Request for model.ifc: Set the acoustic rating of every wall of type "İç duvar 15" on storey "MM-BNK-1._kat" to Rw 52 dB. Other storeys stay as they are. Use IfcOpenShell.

First a look at what the model holds.

```python
import ifcopenshell
import ifcopenshell.util.element

model = ifcopenshell.open("model.ifc")
print(model.schema)
storey = next(s for s in model.by_type("IfcBuildingStorey") if s.Name == "MM-BNK-1._kat")
walls = [e for e in ifcopenshell.util.element.get_decomposition(storey) if e.is_a("IfcWall")]
seen = {}
for e in walls:
    element_type = ifcopenshell.util.element.get_type(e)
    key = (element_type.Name if element_type != e and element_type else None, ifcopenshell.util.element.get_pset(e, "Pset_WallCommon", "AcousticRating"))
    seen[key] = seen.get(key, 0) + 1
for (name, value), count in sorted(seen.items(), key=str):
    print(count, "x", name, "|", value)
```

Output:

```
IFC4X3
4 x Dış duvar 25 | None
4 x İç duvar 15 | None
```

```python
import ifcopenshell
import ifcopenshell.api.pset
import ifcopenshell.util.element

model = ifcopenshell.open("model.ifc")

storey = next(s for s in model.by_type("IfcBuildingStorey") if s.Name == "MM-BNK-1._kat")
walls = [e for e in ifcopenshell.util.element.get_decomposition(storey) if e.is_a("IfcWall")]

count = 0
for e in walls:
    element_type = ifcopenshell.util.element.get_type(e)
    if element_type in (None, e) or element_type.Name != "İç duvar 15":
        continue
    # add_pset returns the element's existing set when there is one.
    pset = ifcopenshell.api.pset.add_pset(model, product=e, name="Pset_WallCommon")
    ifcopenshell.api.pset.edit_pset(model, pset=pset, properties={"AcousticRating": "Rw 52 dB"})
    count += 1

print(count, "walls updated")

model.write("model-out.ifc")
```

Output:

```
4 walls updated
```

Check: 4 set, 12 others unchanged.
